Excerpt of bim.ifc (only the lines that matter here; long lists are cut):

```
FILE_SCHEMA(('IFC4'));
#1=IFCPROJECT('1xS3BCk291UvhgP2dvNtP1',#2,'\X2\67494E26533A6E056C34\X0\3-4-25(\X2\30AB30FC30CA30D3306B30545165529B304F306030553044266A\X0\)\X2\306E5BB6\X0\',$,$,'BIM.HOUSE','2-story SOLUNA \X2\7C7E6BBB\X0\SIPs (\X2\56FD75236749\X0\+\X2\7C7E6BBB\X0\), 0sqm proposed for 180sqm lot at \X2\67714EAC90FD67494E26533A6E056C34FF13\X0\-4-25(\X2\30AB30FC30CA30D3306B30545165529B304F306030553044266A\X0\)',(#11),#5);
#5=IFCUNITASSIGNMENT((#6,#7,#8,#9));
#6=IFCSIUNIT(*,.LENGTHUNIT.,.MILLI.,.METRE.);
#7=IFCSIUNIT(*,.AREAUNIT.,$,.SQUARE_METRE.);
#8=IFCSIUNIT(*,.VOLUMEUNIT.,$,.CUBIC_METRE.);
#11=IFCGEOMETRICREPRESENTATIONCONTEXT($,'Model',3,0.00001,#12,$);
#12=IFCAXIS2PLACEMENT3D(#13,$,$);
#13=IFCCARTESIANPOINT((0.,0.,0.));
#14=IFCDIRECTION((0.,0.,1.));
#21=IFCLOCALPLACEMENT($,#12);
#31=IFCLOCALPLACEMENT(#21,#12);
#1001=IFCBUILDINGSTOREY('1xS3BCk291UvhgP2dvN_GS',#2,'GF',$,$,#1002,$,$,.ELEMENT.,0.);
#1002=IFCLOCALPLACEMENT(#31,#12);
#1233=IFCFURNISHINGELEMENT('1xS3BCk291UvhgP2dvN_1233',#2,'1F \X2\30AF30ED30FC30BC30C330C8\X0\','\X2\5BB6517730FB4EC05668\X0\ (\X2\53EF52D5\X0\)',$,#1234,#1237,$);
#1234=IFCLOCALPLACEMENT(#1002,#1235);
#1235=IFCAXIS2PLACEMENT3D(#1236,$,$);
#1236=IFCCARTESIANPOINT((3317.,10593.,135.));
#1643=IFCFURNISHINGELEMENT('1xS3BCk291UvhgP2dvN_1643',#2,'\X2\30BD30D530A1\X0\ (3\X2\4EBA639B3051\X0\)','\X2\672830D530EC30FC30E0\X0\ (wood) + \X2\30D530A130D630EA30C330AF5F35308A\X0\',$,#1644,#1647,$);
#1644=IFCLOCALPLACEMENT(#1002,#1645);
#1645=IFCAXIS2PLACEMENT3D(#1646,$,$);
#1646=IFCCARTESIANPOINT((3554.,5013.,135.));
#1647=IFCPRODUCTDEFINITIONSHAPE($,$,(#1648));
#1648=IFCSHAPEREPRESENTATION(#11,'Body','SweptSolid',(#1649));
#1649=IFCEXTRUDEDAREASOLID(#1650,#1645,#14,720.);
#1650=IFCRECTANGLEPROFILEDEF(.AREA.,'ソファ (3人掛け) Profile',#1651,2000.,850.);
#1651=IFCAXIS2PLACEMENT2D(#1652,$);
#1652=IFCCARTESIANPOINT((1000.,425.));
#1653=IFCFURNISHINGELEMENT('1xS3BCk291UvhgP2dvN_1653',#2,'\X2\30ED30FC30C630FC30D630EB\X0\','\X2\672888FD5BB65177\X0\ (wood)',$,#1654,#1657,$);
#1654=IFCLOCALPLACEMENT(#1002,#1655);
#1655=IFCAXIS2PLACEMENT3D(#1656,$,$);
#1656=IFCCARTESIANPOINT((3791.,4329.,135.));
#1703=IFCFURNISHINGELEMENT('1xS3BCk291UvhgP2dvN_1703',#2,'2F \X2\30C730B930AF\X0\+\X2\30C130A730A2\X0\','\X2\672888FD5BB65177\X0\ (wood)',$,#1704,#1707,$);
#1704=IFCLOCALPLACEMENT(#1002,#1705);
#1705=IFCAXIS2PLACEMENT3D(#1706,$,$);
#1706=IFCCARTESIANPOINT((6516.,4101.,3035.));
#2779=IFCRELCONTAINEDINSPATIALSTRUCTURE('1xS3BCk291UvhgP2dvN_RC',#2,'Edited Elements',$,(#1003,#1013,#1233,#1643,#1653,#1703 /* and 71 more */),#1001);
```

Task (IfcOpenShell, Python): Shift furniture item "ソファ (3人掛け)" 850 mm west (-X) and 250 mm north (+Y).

```python
import ifcopenshell
import ifcopenshell.api.geometry
import ifcopenshell.util.placement
import ifcopenshell.util.unit

model = ifcopenshell.open("bim.ifc")
unit_scale = ifcopenshell.util.unit.calculate_unit_scale(model)

item = model.by_guid("1xS3BCk291UvhgP2dvN_1643")
matrix = ifcopenshell.util.placement.get_local_placement(item.ObjectPlacement)
matrix[0, 3] -= 0.85 / unit_scale
matrix[1, 3] += 0.25 / unit_scale
ifcopenshell.api.geometry.edit_object_placement(model, product=item, matrix=matrix, is_si=False)

print(ifcopenshell.util.placement.get_local_placement(item.ObjectPlacement).round(3) + 0.0)

model.write("bim_edited.ifc")
```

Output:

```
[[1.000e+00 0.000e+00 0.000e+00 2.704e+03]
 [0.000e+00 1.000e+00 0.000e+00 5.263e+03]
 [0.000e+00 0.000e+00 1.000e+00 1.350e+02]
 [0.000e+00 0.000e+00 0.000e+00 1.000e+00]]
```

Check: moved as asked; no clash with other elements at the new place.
